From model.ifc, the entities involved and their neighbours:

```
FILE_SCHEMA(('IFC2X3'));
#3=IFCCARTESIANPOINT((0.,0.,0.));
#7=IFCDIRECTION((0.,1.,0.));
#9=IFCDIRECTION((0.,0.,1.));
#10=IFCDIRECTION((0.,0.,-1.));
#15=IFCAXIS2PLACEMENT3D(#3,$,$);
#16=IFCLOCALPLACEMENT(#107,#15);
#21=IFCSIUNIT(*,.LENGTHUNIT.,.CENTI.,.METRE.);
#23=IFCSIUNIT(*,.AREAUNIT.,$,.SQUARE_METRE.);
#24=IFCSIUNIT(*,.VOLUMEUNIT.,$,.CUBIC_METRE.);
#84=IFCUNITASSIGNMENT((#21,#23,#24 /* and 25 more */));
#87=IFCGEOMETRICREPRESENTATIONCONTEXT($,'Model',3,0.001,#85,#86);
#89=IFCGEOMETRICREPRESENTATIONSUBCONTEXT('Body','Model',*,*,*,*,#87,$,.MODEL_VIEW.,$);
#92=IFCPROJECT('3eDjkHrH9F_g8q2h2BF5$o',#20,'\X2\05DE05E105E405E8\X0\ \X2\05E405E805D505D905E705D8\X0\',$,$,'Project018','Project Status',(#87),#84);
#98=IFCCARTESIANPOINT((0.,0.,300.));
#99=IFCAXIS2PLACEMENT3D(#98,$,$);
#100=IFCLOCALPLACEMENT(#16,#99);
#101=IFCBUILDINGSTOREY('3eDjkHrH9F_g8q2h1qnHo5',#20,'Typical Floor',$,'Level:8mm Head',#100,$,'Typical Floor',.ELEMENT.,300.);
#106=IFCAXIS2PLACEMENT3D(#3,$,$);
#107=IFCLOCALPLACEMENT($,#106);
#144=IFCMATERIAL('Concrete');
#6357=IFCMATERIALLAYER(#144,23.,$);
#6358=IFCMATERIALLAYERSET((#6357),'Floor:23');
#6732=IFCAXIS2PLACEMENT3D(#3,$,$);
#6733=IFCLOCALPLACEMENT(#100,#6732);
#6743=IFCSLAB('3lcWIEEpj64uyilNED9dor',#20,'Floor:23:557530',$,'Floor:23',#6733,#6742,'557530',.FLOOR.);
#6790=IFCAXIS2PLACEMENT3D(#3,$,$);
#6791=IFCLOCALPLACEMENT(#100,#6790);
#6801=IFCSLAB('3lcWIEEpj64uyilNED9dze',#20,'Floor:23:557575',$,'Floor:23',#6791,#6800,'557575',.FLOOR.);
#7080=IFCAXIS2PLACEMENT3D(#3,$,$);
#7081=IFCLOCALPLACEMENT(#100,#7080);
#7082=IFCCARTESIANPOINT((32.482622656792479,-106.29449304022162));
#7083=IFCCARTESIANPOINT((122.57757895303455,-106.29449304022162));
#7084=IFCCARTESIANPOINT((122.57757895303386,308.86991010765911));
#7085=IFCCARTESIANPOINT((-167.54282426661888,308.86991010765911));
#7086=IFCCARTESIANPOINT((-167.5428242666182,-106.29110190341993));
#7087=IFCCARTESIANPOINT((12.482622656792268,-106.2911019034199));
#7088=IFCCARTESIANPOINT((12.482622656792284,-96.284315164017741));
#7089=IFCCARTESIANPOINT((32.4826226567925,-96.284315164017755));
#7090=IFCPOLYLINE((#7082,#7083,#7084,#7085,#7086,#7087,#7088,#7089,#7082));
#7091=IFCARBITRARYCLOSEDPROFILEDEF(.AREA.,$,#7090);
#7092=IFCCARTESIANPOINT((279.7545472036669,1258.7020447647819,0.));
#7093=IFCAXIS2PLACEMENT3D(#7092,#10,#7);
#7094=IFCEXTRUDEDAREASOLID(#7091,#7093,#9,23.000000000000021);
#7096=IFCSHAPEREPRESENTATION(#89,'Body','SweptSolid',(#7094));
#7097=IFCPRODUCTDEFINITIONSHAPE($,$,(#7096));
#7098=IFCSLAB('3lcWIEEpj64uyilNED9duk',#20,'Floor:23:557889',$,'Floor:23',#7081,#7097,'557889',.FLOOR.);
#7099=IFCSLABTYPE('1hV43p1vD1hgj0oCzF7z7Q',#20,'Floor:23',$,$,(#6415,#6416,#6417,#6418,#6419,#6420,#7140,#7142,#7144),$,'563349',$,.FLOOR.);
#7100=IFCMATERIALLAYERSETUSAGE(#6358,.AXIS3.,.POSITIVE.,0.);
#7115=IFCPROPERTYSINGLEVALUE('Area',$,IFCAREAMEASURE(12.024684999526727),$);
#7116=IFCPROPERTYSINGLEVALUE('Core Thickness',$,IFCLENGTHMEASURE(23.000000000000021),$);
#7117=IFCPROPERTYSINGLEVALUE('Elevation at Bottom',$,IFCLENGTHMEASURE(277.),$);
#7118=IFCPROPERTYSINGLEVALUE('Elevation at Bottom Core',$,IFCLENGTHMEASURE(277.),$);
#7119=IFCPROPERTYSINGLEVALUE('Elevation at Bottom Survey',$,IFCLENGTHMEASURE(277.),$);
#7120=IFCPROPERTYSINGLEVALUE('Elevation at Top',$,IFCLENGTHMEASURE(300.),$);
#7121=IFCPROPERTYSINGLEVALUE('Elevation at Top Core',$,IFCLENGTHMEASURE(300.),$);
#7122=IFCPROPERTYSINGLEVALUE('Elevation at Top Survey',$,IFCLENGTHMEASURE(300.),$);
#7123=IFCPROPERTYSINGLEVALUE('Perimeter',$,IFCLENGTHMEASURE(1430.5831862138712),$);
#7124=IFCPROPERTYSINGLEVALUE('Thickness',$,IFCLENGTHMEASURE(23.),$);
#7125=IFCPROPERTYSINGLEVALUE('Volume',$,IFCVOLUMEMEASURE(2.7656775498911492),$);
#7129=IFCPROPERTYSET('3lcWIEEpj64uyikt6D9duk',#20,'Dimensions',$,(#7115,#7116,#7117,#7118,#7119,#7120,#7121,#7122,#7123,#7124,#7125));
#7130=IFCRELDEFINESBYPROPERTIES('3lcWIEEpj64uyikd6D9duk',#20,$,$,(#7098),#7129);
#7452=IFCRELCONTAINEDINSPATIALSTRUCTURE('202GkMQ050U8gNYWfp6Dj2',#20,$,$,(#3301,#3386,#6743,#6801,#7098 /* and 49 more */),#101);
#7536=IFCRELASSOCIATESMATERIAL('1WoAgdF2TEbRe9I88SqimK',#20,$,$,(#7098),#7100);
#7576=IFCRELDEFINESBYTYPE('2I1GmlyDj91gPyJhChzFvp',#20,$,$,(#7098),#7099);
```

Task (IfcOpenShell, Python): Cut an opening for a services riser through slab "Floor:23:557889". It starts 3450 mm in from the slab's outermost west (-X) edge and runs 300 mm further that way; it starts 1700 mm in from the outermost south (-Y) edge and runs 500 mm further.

```python
import numpy as np
import ifcopenshell
import ifcopenshell.api.feature
import ifcopenshell.api.geometry
import ifcopenshell.api.pset
import ifcopenshell.api.root
import ifcopenshell.geom
import ifcopenshell.util.element
import ifcopenshell.util.placement
import ifcopenshell.util.representation
import ifcopenshell.util.shape
import ifcopenshell.util.unit

model = ifcopenshell.open("model.ifc")
unit_scale = ifcopenshell.util.unit.calculate_unit_scale(model)
area_scale = ifcopenshell.util.unit.calculate_unit_scale(model, "AREAUNIT")
volume_scale = ifcopenshell.util.unit.calculate_unit_scale(model, "VOLUMEUNIT")
settings = ifcopenshell.geom.settings()


def volume(element):
    """Net volume in cubic metres, openings subtracted."""
    shape = ifcopenshell.geom.create_shape(settings, element)
    return ifcopenshell.util.shape.get_volume(shape.geometry)


slab = model.by_guid("3lcWIEEpj64uyilNED9duk")
before = volume(slab)

# Extent in the slab's own axes, in metres. The edges named are its -X and -Y sides.
slab_shape = ifcopenshell.geom.create_shape(settings, slab)
vertices = ifcopenshell.util.shape.get_vertices(slab_shape.geometry)
x_min, y_min, bottom = vertices.min(axis=0)
top = vertices[:, 2].max()

opening = ifcopenshell.api.root.create_entity(model, ifc_class="IfcOpeningElement", name="Services riser opening")
context = ifcopenshell.util.representation.get_context(model, "Model", "Body", "MODEL_VIEW")
width, depth = 0.3, 0.5
outline = [(0.0, 0.0), (width, 0.0), (width, depth), (0.0, depth), (0.0, 0.0)]
# Overshoot both faces by 50 mm so the cut is clean.
shape = ifcopenshell.api.geometry.add_slab_representation(
    model, context=context, depth=top - bottom + 0.1, polyline=outline
)
ifcopenshell.api.geometry.assign_representation(model, product=opening, representation=shape)

matrix = ifcopenshell.util.placement.get_local_placement(slab.ObjectPlacement)
matrix[:, 3] = matrix @ np.append(np.array([x_min + 3.45, y_min + 1.7, bottom - 0.05]) / unit_scale, 1.0)
ifcopenshell.api.geometry.edit_object_placement(model, product=opening, matrix=matrix, is_si=False)
ifcopenshell.api.feature.add_feature(model, feature=opening, element=slab)

after = volume(slab)

# Update the slab's stored quantities.
pset = model.by_id(ifcopenshell.util.element.get_pset(slab, "Dimensions", should_inherit=False)["id"])
ifcopenshell.api.pset.edit_pset(model, pset=pset, properties={
    "Area": model.create_entity("IfcAreaMeasure", after / (top - bottom) / area_scale),
    "Volume": model.create_entity("IfcVolumeMeasure", after / volume_scale),
})

print(f"slab volume {before:.3f} -> {after:.3f} m3")

model.write("model-out.ifc")
```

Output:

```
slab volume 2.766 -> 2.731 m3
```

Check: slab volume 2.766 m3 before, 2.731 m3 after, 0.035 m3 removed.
